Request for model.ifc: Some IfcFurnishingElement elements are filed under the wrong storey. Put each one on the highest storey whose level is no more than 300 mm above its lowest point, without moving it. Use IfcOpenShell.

First a look at what the model holds.

```python
import ifcopenshell
import ifcopenshell.util.element
import ifcopenshell.util.placement

model = ifcopenshell.open("model.ifc")
print(model.schema)
for storey in model.by_type("IfcBuildingStorey"):
    level = ifcopenshell.util.placement.get_storey_elevation(storey)
    count = sum(e.is_a("IfcFurnishingElement") for e in ifcopenshell.util.element.get_contained(storey))
    print(storey.id(), storey.Name, round(level, 3), count, sep=" | ")
```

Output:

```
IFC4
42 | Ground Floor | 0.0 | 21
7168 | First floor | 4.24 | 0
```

```python
import ifcopenshell
import ifcopenshell.api.spatial
import ifcopenshell.geom
import ifcopenshell.util.element
import ifcopenshell.util.placement
import ifcopenshell.util.shape
import ifcopenshell.util.unit

model = ifcopenshell.open("model.ifc")
unit_scale = ifcopenshell.util.unit.calculate_unit_scale(model)
settings = ifcopenshell.geom.settings()

levels = sorted(
    ((ifcopenshell.util.placement.get_storey_elevation(s) * unit_scale, s) for s in model.by_type("IfcBuildingStorey")),
    key=lambda pair: pair[0],
)

for e in model.by_type("IfcFurnishingElement"):
    current = e.ContainedInStructure[0].RelatingStructure if e.ContainedInStructure else None
    if current is None or not current.is_a("IfcBuildingStorey"):
        continue
    shape = ifcopenshell.geom.create_shape(settings, e)
    bottom = ifcopenshell.util.shape.get_shape_bottom_elevation(shape, shape.geometry)
    below = [s for level, s in levels if level <= bottom + 0.3]
    storey = below[-1] if below else levels[0][1]
    if storey != current:
        # assign_container keeps the world position.
        ifcopenshell.api.spatial.assign_container(model, products=[e], relating_structure=storey)
        print(e.id(), current.Name, "->", storey.Name)

model.write("model_updated.ifc")
```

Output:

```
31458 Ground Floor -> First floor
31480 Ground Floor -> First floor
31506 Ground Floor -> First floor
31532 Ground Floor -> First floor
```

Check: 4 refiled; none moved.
